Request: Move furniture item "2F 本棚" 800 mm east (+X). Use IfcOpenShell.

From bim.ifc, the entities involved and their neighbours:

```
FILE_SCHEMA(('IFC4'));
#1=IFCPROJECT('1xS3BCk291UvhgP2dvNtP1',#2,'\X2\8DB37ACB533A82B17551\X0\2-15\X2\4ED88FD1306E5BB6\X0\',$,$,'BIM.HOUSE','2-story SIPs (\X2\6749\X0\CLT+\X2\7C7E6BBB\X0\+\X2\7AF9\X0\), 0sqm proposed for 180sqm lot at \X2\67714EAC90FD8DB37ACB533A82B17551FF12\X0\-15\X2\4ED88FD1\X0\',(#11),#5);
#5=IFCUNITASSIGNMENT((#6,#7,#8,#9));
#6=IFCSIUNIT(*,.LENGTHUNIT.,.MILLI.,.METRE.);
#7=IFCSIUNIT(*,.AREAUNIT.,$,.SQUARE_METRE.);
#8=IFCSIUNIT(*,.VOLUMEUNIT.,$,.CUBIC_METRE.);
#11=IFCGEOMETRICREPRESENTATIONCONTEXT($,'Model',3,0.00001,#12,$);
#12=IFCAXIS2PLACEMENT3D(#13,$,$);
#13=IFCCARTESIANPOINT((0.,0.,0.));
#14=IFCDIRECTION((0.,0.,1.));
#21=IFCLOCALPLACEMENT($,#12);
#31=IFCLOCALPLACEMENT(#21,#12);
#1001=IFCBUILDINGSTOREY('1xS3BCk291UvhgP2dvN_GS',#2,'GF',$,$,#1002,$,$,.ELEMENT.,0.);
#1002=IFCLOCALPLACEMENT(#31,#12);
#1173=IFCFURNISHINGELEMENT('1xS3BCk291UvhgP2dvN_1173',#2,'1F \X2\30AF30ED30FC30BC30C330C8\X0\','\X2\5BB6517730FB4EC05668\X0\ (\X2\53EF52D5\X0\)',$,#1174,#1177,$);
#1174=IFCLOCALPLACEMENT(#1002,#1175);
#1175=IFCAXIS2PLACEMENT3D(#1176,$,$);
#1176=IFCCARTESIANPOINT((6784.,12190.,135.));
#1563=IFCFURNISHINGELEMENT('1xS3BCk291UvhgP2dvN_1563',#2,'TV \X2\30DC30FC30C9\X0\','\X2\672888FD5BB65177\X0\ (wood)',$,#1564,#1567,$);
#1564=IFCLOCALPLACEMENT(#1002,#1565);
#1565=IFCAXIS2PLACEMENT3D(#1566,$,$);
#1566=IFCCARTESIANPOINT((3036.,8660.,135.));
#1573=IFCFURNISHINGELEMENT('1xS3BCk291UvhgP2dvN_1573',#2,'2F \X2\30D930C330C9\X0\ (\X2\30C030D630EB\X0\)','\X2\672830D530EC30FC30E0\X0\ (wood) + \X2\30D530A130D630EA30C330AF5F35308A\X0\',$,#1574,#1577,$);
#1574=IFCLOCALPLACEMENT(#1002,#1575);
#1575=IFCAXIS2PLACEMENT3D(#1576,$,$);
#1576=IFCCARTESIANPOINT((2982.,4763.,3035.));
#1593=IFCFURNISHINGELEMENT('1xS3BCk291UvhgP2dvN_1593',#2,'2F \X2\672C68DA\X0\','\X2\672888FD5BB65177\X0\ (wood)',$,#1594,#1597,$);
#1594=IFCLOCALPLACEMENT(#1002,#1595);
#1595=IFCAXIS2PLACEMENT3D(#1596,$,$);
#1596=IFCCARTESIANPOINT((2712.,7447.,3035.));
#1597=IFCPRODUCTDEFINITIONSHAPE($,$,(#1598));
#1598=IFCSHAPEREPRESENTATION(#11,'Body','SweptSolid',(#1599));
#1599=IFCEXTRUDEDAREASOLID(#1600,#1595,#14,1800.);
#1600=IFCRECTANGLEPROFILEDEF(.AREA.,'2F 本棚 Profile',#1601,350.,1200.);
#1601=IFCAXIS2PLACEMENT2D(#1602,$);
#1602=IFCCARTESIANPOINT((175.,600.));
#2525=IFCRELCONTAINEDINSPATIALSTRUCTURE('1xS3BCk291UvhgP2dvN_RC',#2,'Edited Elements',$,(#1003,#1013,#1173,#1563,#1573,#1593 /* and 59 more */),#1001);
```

```python
import ifcopenshell
import ifcopenshell.api.geometry
import ifcopenshell.util.placement
import ifcopenshell.util.unit

model = ifcopenshell.open("bim.ifc")
unit_scale = ifcopenshell.util.unit.calculate_unit_scale(model)

item = model.by_id(1593)
matrix = ifcopenshell.util.placement.get_local_placement(item.ObjectPlacement)
matrix[0, 3] += 0.8 / unit_scale
ifcopenshell.api.geometry.edit_object_placement(model, product=item, matrix=matrix, is_si=False)

print(ifcopenshell.util.placement.get_local_placement(item.ObjectPlacement).round(3) + 0.0)

model.write("bim_updated.ifc")
```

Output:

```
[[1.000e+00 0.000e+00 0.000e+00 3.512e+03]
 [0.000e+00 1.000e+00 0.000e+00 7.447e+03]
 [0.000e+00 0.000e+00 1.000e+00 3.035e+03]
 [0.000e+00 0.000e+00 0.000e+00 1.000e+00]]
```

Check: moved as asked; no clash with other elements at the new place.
